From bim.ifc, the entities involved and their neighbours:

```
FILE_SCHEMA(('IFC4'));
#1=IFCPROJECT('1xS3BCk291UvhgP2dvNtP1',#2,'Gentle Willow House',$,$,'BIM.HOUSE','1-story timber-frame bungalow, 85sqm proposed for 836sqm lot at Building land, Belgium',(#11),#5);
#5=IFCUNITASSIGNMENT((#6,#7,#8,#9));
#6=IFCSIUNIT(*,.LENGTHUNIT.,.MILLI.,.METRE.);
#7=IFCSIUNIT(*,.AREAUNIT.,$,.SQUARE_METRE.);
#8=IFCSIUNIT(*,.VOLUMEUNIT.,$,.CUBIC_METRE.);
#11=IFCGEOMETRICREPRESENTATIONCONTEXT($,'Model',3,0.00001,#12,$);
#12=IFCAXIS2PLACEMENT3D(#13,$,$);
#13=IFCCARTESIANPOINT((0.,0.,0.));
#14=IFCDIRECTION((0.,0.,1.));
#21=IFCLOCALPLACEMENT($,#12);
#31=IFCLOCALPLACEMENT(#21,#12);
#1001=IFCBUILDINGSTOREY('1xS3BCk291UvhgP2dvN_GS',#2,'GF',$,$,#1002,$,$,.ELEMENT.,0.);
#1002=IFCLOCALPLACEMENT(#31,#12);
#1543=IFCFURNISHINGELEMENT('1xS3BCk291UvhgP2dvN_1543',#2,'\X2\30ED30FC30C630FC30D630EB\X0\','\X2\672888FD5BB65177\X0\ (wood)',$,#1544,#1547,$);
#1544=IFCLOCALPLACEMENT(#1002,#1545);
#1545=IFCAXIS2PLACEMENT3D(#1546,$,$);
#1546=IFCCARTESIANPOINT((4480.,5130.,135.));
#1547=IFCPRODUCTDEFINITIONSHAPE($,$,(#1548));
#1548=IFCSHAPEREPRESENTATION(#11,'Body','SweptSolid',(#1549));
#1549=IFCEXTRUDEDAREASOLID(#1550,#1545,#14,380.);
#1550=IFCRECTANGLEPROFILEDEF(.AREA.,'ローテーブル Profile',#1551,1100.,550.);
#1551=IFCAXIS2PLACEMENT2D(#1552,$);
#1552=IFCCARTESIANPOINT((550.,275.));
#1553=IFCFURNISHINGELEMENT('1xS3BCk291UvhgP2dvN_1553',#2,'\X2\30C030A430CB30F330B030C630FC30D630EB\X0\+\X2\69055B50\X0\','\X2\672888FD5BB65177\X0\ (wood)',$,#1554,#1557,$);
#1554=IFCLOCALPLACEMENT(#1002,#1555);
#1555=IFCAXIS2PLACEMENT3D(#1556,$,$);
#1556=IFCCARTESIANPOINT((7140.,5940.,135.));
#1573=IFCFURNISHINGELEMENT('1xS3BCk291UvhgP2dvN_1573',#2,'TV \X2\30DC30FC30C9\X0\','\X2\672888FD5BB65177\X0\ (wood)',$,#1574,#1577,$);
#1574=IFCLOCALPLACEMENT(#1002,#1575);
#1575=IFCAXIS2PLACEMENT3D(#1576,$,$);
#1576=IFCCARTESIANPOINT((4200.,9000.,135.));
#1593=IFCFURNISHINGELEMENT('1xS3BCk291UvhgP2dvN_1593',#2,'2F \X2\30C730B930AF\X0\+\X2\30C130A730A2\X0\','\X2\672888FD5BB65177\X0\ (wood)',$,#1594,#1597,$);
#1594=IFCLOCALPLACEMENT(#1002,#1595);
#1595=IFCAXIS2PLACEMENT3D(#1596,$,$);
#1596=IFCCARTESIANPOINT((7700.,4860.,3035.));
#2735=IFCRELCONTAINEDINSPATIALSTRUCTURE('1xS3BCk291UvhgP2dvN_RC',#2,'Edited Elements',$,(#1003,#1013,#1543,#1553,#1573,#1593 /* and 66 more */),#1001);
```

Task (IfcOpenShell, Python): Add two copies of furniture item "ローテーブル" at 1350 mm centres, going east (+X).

```python
import numpy as np
import ifcopenshell
import ifcopenshell.api.geometry
import ifcopenshell.api.root
import ifcopenshell.util.element
import ifcopenshell.util.placement
import ifcopenshell.util.unit

model = ifcopenshell.open("bim.ifc")
unit_scale = ifcopenshell.util.unit.calculate_unit_scale(model)


def reuse_history(source, copy):
    """copy_class also copies each property set's owner history, people and application; keep the originals."""
    for rel in copy.IsDefinedBy:
        if rel.is_a("IfcRelDefinesByProperties") and (history := rel.RelatingPropertyDefinition.OwnerHistory):
            rel.RelatingPropertyDefinition.OwnerHistory = source.OwnerHistory
            ifcopenshell.util.element.remove_deep2(model, history)


source = model.by_id(1543)
base = ifcopenshell.util.placement.get_local_placement(source.ObjectPlacement)
step = np.array([1.0, 0.0, 0.0]) * 1.35 / unit_scale

for i in range(1, 3):
    copy = ifcopenshell.api.root.copy_class(model, product=source)
    copy.Representation = ifcopenshell.util.element.copy_deep(
        model, source.Representation, exclude=["IfcGeometricRepresentationContext", "IfcRepresentationMap"]
    )
    reuse_history(source, copy)
    matrix = base.copy()
    matrix[:3, 3] += i * step
    print("added at", matrix[:3, 3].round(3) + 0.0)
    ifcopenshell.api.geometry.edit_object_placement(model, product=copy, matrix=matrix, is_si=False)

model.write("bim-out.ifc")
```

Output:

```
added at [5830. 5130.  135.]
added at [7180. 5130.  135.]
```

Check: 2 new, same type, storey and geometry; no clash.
